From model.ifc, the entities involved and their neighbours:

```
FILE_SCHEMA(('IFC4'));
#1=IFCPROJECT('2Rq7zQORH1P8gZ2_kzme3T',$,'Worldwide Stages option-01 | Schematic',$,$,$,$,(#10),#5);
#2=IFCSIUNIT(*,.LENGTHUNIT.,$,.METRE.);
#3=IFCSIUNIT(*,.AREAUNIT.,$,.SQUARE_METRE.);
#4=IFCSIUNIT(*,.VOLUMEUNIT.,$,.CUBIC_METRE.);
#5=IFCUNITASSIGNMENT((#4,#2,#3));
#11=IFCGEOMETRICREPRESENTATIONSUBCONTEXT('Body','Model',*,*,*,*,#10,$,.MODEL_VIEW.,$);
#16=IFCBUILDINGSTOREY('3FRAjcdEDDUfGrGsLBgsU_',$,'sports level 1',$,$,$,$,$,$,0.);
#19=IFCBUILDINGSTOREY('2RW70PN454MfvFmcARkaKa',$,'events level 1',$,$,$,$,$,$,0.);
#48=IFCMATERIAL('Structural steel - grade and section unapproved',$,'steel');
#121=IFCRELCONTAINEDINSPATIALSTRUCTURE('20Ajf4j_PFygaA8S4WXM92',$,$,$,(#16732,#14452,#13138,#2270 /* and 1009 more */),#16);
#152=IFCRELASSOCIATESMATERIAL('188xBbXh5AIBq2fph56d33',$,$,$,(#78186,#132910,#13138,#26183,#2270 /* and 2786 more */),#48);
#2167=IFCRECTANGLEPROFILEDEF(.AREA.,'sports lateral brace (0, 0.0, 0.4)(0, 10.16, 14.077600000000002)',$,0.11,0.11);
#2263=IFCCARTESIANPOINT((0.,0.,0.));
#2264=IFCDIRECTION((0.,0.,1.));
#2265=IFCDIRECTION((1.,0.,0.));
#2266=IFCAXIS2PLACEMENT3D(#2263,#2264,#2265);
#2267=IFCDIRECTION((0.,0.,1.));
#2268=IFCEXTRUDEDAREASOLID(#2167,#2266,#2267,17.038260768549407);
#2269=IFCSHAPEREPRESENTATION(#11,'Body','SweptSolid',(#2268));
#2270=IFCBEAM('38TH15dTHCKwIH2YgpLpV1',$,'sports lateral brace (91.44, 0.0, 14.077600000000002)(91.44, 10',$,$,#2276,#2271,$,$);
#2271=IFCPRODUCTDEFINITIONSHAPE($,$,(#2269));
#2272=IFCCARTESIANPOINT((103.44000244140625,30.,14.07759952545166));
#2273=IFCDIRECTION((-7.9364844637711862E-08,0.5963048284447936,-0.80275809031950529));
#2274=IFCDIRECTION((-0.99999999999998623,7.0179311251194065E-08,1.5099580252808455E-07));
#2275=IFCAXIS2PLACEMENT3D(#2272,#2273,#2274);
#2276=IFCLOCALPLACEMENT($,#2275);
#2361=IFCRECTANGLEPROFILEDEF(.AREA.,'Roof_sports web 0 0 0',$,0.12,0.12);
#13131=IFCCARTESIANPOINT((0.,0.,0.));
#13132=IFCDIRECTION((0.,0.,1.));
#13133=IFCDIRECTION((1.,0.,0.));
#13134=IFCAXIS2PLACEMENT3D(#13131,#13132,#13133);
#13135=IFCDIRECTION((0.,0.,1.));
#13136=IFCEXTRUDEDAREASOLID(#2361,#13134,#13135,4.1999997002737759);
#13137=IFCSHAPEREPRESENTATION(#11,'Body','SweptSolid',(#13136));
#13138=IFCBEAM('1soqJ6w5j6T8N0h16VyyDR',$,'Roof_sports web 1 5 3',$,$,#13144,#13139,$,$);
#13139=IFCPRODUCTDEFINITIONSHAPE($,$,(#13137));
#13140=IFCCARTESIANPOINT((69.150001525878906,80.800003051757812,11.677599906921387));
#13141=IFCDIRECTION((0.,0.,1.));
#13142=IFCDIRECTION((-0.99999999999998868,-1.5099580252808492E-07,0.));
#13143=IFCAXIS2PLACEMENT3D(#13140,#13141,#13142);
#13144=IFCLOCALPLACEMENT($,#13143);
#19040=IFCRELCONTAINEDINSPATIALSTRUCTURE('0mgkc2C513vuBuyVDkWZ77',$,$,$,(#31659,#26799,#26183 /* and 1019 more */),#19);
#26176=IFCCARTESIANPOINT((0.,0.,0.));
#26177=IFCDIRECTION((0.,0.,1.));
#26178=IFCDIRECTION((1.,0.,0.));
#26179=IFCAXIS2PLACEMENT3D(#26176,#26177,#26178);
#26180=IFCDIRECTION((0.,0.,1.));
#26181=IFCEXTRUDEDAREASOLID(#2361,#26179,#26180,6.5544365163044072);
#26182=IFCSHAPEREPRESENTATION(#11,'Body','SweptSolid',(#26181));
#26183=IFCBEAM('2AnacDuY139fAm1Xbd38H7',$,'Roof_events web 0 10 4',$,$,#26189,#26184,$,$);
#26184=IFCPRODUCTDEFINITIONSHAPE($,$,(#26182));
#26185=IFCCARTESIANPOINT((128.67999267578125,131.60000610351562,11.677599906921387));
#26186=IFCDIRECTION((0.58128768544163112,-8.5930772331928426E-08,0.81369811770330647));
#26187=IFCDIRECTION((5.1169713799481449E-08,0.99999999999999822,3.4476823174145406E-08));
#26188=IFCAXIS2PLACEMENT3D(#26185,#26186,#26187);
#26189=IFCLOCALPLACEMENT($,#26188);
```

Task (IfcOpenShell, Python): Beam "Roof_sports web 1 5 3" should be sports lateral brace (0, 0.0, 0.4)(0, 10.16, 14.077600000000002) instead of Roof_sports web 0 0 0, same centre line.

```python
import ifcopenshell
import ifcopenshell.util.element
import ifcopenshell.util.representation

model = ifcopenshell.open("model.ifc")

member = model.by_id(13138)
source = next(p for p in model.by_type("IfcRectangleProfileDef") if p.ProfileName == "sports lateral brace (0, 0.0, 0.4)(0, 10.16, 14.077600000000002)")

body = ifcopenshell.util.representation.get_representation(member, "Model", "Body")
solid = body.Items[0]
old_profile = solid.SweptArea

# Copy the section's sizes but keep this member's own profile position.
profile = ifcopenshell.util.element.copy(model, source)
profile.Position = old_profile.Position
solid.SweptArea = profile
if not model.get_total_inverses(old_profile):
    ifcopenshell.util.element.remove_deep2(model, old_profile)

print(solid.SweptArea)

model.write("model_updated.ifc")
```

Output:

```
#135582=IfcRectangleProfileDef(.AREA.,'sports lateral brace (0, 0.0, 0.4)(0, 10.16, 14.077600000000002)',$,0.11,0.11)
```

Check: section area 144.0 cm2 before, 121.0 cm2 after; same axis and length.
